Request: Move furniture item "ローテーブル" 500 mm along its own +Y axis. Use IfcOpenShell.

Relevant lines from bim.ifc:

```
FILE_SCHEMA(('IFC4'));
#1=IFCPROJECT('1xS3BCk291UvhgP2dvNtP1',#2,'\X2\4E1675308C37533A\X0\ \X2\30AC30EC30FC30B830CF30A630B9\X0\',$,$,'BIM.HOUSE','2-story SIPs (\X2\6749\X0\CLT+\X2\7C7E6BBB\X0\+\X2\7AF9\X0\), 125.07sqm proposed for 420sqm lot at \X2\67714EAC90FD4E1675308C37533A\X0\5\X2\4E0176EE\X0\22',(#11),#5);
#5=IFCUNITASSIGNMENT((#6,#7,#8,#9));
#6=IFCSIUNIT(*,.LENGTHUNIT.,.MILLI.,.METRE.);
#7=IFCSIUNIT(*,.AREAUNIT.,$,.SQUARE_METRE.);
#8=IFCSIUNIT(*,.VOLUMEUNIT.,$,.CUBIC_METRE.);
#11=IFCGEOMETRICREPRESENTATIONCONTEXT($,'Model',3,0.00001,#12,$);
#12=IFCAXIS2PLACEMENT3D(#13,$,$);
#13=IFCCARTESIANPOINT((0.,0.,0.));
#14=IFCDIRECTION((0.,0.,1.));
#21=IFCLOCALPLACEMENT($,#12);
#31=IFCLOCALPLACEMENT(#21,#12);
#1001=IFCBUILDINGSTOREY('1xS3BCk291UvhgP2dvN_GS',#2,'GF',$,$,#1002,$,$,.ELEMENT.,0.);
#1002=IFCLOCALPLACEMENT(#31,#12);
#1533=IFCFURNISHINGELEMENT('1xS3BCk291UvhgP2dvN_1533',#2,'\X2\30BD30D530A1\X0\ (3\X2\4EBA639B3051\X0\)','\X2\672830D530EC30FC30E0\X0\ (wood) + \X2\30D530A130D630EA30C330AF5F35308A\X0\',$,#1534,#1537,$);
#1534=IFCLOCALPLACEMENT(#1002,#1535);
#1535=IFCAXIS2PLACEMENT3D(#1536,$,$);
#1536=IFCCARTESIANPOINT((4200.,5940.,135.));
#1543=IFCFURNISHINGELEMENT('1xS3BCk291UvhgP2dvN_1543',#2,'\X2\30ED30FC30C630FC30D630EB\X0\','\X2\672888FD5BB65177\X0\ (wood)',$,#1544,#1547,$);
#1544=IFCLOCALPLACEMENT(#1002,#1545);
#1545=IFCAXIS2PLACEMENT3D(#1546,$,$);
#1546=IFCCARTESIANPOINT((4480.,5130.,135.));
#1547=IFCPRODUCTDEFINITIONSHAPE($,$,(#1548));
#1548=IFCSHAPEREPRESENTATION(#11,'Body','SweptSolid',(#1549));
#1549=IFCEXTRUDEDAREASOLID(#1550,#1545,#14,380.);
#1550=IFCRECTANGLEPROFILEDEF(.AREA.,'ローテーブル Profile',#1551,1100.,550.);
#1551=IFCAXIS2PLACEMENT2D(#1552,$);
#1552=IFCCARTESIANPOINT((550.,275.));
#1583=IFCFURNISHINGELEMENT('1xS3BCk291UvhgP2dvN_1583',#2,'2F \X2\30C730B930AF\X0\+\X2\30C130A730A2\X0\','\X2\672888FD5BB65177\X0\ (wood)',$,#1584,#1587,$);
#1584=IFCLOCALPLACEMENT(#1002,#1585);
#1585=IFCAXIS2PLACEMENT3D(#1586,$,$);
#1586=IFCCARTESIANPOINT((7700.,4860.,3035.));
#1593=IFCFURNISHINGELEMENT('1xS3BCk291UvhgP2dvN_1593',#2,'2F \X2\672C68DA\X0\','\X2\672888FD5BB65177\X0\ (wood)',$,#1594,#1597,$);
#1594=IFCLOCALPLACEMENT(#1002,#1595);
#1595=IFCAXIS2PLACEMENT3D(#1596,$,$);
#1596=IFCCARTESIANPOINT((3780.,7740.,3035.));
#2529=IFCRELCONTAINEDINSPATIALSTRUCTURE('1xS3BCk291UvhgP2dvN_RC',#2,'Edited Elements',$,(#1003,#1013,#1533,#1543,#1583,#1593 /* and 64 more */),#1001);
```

```python
import ifcopenshell
import ifcopenshell.api.geometry
import ifcopenshell.util.placement
import ifcopenshell.util.unit

model = ifcopenshell.open("bim.ifc")
unit_scale = ifcopenshell.util.unit.calculate_unit_scale(model)

item = model.by_id(1543)
matrix = ifcopenshell.util.placement.get_local_placement(item.ObjectPlacement)
matrix[:3, 3] += matrix[:3, 1] * 0.5 / unit_scale
ifcopenshell.api.geometry.edit_object_placement(model, product=item, matrix=matrix, is_si=False)

print(ifcopenshell.util.placement.get_local_placement(item.ObjectPlacement).round(3) + 0.0)

model.write("bim_v2.ifc")
```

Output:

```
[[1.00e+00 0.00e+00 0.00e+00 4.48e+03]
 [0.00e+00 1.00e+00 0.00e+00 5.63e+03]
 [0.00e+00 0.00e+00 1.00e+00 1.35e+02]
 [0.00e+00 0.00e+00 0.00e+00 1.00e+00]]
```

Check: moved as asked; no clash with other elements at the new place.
